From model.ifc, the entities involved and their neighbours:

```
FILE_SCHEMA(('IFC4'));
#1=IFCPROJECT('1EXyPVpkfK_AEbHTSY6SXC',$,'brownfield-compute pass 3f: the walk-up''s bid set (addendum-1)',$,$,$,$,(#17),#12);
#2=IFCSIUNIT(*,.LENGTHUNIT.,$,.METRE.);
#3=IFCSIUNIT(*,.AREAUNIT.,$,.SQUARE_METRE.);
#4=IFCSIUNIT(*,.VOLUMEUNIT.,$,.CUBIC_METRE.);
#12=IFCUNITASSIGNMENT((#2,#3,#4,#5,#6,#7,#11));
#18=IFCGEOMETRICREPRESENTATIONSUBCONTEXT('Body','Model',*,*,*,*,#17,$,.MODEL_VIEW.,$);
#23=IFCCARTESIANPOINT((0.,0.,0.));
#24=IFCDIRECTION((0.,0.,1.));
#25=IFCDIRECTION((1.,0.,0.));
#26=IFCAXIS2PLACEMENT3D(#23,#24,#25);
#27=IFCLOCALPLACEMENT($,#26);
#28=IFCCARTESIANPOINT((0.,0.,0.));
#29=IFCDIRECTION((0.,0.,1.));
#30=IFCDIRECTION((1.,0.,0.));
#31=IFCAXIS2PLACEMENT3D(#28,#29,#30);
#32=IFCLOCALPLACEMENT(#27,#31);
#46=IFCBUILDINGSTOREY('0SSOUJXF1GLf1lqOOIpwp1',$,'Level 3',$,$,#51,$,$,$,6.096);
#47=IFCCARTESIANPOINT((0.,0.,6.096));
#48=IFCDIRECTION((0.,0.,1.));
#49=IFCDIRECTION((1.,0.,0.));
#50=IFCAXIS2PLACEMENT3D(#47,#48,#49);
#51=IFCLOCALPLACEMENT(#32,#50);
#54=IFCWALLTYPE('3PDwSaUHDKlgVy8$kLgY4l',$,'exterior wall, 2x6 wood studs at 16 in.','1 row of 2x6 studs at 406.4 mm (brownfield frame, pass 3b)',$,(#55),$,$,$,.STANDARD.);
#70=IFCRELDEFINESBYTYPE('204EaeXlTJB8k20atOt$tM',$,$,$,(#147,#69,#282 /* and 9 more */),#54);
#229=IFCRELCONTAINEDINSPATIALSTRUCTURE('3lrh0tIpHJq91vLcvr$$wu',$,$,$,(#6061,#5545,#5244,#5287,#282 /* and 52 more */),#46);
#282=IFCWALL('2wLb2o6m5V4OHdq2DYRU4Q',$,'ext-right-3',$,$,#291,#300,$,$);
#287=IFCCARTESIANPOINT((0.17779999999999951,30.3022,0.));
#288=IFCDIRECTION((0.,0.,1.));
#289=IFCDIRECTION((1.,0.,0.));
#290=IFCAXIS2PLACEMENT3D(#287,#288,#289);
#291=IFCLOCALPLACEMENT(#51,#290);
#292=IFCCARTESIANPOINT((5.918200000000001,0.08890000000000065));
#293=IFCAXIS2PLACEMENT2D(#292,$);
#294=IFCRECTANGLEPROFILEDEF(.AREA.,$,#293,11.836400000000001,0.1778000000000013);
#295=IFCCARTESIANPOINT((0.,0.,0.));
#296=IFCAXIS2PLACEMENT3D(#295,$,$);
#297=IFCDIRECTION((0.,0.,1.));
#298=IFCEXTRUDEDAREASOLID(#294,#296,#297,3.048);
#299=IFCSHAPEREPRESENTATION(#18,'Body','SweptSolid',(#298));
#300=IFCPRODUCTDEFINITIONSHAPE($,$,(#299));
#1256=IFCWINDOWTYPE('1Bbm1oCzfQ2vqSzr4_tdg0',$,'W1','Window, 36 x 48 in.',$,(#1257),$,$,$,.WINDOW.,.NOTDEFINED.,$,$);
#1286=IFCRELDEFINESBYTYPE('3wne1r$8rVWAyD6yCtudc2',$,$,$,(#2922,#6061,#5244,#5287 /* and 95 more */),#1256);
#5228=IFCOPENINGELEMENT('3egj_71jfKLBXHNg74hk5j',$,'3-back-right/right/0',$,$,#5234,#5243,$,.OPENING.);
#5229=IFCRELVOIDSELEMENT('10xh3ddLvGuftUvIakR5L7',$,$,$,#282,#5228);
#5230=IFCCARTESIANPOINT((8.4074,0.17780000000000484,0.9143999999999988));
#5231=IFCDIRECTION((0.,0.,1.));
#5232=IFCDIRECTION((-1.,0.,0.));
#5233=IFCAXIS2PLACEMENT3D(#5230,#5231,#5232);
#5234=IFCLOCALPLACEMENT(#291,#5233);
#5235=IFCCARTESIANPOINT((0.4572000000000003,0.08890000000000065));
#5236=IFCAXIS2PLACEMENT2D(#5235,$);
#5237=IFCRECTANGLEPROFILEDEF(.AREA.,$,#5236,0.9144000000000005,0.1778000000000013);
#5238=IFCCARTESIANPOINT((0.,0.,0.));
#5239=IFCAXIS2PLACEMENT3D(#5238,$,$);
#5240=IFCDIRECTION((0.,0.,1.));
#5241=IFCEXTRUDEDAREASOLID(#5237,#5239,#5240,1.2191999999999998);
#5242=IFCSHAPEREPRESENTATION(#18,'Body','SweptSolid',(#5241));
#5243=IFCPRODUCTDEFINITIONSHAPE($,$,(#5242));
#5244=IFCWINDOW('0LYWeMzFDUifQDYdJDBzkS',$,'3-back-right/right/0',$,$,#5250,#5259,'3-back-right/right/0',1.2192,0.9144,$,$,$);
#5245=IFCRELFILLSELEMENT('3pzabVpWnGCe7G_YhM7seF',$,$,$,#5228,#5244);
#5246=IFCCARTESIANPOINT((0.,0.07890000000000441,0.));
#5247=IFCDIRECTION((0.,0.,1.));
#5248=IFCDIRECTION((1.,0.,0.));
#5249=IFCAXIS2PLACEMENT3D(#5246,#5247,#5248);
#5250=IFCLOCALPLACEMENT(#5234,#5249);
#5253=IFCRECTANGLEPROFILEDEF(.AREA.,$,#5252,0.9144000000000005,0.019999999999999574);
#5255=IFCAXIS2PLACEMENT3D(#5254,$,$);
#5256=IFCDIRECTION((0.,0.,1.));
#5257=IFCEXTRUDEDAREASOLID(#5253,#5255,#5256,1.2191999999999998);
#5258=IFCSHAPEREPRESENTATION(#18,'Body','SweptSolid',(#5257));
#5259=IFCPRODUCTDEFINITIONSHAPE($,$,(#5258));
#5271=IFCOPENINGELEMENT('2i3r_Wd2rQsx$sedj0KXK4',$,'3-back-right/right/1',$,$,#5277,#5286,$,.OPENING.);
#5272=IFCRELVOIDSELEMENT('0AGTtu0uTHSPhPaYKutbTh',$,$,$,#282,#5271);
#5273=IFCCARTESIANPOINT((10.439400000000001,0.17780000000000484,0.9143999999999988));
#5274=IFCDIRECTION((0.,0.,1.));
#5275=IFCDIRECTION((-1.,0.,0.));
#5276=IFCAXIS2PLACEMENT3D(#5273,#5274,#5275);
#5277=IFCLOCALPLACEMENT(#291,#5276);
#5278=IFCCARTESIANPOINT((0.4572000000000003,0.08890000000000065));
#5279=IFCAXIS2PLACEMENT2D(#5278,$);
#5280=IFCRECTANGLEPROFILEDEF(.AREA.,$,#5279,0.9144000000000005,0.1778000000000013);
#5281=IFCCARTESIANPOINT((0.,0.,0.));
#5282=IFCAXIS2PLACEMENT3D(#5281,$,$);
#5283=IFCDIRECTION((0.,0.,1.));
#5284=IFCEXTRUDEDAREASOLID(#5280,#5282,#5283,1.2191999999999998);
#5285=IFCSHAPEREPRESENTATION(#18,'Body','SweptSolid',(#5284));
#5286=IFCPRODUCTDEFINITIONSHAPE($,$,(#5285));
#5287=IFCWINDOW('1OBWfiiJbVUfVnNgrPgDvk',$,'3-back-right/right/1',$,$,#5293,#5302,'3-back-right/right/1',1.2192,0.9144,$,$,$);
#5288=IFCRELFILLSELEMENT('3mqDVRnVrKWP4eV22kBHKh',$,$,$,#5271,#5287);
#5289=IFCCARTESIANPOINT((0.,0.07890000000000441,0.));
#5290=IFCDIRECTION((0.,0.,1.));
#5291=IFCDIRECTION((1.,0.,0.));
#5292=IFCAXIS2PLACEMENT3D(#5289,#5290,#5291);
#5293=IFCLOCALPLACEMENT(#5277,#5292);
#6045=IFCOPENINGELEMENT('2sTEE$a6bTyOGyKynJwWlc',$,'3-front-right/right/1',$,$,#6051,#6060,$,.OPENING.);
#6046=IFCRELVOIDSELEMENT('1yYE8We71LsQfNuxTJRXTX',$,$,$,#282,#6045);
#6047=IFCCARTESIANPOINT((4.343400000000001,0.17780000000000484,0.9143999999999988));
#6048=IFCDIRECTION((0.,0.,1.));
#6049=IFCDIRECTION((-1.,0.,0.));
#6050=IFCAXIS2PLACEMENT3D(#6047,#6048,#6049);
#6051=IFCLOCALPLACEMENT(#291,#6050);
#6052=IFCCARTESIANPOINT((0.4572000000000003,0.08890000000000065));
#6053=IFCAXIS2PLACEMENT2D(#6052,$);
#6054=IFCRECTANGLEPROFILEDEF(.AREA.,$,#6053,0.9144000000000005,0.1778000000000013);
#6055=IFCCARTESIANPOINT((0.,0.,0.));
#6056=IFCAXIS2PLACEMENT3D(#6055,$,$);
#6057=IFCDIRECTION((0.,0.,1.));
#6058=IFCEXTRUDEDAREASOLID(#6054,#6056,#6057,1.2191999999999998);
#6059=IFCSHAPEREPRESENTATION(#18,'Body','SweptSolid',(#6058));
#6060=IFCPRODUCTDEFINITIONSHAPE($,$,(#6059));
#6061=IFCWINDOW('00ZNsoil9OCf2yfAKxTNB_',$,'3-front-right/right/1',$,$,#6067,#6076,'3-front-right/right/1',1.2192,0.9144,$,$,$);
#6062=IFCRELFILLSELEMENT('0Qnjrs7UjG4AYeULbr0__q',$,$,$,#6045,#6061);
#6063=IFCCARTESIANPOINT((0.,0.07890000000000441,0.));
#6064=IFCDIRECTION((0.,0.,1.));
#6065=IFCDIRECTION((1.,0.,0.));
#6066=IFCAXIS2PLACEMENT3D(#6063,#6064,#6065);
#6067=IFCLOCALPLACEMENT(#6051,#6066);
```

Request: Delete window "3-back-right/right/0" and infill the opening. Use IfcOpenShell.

```python
import ifcopenshell
import ifcopenshell.api.feature
import ifcopenshell.api.root
import ifcopenshell.geom
import ifcopenshell.util.shape

model = ifcopenshell.open("model.ifc")
settings = ifcopenshell.geom.settings()


def volume(element):
    """Net volume in cubic metres, openings subtracted."""
    shape = ifcopenshell.geom.create_shape(settings, element)
    return ifcopenshell.util.shape.get_volume(shape.geometry)


window = model.by_id(5244)
opening = window.FillsVoids[0].RelatingOpeningElement
wall = opening.VoidsElements[0].RelatingBuildingElement
before = volume(wall)

ifcopenshell.api.root.remove_product(model, product=window)
ifcopenshell.api.feature.remove_feature(model, feature=opening)

after = volume(wall)

print(f"wall volume {before:.3f} -> {after:.3f} m3")

model.write("model-out.ifc")
```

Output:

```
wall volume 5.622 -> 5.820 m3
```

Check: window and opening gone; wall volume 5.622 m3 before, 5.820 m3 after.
